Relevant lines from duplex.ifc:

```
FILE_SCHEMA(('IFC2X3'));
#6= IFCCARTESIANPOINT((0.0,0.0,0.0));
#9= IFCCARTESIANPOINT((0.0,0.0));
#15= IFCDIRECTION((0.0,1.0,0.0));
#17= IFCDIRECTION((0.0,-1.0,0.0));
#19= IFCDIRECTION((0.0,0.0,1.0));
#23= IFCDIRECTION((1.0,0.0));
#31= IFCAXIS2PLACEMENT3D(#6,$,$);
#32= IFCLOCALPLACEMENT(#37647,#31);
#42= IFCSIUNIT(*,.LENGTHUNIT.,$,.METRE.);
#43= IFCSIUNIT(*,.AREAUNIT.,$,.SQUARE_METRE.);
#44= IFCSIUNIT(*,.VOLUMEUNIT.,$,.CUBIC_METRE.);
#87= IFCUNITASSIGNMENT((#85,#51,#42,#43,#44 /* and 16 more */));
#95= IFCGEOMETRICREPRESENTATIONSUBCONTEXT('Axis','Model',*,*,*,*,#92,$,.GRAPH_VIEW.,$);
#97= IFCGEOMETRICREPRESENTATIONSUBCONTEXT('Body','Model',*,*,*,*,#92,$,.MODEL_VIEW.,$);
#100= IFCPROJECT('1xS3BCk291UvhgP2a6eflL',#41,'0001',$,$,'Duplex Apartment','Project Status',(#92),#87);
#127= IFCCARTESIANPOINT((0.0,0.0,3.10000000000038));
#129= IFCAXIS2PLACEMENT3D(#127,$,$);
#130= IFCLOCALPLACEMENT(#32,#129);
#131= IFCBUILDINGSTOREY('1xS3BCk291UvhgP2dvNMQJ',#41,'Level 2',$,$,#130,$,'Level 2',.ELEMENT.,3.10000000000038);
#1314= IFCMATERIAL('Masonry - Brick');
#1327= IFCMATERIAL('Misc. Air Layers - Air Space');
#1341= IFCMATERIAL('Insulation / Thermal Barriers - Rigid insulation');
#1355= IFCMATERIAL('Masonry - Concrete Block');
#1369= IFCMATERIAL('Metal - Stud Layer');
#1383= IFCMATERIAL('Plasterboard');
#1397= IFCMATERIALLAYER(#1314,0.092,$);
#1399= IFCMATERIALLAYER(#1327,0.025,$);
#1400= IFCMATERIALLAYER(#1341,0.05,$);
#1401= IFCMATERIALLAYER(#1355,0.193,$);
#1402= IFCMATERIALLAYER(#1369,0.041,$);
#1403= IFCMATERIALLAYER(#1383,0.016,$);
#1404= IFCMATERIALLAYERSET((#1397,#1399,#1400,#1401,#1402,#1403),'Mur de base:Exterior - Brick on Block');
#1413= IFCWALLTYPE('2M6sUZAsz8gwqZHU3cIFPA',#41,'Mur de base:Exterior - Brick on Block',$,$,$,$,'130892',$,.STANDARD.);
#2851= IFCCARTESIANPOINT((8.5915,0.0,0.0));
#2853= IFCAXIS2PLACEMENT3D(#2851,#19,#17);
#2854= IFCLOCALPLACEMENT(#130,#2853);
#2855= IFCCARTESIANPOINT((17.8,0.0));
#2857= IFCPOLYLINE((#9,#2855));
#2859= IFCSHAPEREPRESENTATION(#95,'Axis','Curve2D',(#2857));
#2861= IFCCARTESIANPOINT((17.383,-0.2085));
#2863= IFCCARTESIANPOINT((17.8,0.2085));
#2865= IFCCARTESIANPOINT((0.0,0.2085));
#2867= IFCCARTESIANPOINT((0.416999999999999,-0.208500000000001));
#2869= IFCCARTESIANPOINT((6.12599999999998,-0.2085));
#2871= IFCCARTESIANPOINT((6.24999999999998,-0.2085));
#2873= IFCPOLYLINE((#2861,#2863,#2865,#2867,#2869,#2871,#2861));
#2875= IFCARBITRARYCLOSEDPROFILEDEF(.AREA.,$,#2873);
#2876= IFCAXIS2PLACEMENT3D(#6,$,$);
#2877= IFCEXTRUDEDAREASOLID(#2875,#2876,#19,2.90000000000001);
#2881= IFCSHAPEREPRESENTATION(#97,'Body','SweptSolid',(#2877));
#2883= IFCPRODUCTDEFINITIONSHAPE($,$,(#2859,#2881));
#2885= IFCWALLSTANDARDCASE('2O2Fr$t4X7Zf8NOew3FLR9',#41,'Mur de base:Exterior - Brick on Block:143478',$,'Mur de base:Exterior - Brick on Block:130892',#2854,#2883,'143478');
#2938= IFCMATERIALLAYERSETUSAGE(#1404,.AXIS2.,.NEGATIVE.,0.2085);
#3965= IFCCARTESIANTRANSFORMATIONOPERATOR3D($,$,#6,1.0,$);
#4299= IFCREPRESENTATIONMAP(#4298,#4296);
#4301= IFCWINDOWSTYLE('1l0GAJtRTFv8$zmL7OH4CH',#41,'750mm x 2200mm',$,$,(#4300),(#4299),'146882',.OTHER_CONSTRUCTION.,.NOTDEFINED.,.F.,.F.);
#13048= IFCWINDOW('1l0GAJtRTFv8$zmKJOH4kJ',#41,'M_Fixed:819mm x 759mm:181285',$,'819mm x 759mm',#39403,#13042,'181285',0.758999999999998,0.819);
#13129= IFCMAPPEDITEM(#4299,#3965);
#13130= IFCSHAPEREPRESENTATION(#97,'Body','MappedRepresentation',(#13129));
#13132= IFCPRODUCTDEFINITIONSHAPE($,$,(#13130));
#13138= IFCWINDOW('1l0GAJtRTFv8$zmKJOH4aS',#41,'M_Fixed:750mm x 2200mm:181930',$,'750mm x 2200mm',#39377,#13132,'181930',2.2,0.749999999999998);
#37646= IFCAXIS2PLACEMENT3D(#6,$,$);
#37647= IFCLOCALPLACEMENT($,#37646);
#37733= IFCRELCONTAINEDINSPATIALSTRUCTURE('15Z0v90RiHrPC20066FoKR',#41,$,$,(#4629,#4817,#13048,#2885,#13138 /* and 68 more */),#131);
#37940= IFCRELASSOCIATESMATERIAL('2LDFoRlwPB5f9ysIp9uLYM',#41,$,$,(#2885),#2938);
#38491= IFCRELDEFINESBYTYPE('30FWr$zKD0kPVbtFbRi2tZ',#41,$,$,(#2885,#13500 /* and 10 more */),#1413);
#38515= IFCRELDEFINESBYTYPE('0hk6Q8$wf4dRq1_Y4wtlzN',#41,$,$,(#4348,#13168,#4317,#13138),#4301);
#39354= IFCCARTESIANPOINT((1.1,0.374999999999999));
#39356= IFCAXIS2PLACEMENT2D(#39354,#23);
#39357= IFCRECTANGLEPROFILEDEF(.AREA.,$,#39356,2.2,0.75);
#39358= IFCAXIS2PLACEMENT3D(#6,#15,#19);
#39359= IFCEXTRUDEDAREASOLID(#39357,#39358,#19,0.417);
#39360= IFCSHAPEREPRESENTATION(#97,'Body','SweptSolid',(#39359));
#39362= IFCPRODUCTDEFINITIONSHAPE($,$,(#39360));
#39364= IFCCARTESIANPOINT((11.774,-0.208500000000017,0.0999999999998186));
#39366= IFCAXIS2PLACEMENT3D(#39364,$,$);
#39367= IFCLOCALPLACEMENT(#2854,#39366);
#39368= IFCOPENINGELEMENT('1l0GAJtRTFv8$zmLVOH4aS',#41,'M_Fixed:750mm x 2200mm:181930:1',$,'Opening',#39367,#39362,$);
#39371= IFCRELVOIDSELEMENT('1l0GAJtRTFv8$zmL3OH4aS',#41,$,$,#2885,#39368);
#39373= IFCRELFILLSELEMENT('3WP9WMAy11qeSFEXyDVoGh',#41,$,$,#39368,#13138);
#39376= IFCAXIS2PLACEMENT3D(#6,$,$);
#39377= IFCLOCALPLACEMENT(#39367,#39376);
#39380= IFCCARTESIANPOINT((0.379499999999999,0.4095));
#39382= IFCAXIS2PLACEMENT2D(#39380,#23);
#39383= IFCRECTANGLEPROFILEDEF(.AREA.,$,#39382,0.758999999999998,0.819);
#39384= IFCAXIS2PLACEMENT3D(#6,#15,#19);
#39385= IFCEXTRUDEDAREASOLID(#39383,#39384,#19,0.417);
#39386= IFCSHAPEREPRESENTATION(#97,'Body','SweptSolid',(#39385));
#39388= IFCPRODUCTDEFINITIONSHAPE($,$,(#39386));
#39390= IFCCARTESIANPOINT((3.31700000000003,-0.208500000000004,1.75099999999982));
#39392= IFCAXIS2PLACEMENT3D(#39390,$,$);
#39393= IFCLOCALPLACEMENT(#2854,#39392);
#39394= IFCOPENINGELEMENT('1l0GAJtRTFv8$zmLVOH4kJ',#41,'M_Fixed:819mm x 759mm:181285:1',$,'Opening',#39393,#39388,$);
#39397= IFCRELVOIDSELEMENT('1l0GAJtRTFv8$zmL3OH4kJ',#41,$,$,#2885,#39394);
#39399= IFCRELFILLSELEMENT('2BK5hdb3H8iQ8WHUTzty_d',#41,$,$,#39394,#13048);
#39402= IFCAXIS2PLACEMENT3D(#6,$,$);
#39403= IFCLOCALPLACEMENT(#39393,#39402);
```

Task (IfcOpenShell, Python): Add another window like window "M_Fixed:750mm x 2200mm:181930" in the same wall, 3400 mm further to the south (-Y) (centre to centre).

```python
import ifcopenshell
import ifcopenshell.api.feature
import ifcopenshell.api.geometry
import ifcopenshell.api.root
import ifcopenshell.geom
import ifcopenshell.util.element
import ifcopenshell.util.placement
import ifcopenshell.util.shape

model = ifcopenshell.open("duplex.ifc")
settings = ifcopenshell.geom.settings()


def volume(element):
    """Net volume in cubic metres, openings subtracted."""
    shape = ifcopenshell.geom.create_shape(settings, element)
    return ifcopenshell.util.shape.get_volume(shape.geometry)


def reuse_history(source, copy):
    """copy_class also copies each property set's owner history, people and application; keep the originals."""
    for rel in copy.IsDefinedBy:
        if rel.is_a("IfcRelDefinesByProperties") and (history := rel.RelatingPropertyDefinition.OwnerHistory):
            rel.RelatingPropertyDefinition.OwnerHistory = source.OwnerHistory
            ifcopenshell.util.element.remove_deep2(model, history)


window = model.by_guid("1l0GAJtRTFv8$zmKJOH4aS")
opening = window.FillsVoids[0].RelatingOpeningElement
wall = opening.VoidsElements[0].RelatingBuildingElement
before = volume(wall)
shift = ifcopenshell.util.placement.get_local_placement(wall.ObjectPlacement)[:3, 0] * 3.4

# copy_class copies the void relationship, type, container and properties, but no geometry.
new_opening = ifcopenshell.api.root.copy_class(model, product=opening)
new_opening.Representation = ifcopenshell.util.element.copy_deep(
    model, opening.Representation, exclude=["IfcGeometricRepresentationContext", "IfcRepresentationMap"]
)
new_opening.Name = "M_Fixed:750mm x 2200mm"
new_window = ifcopenshell.api.root.copy_class(model, product=window)
new_window.Representation = ifcopenshell.util.element.copy_deep(
    model, window.Representation, exclude=["IfcGeometricRepresentationContext", "IfcRepresentationMap"]
)
new_window.Name = "M_Fixed:750mm x 2200mm"
new_window.Tag = None
reuse_history(window, new_window)
fills = ifcopenshell.api.feature.add_filling(model, opening=new_opening, element=new_window)
fills.OwnerHistory = new_window.OwnerHistory  # required in IFC2X3

for old, new in ((opening, new_opening), (window, new_window)):
    matrix = ifcopenshell.util.placement.get_local_placement(old.ObjectPlacement)
    matrix[:3, 3] += shift
    ifcopenshell.api.geometry.edit_object_placement(model, product=new, matrix=matrix, is_si=False)

after = volume(wall)

print(f"wall volume {before:.3f} -> {after:.3f} m3")

model.write("duplex_edited.ifc")
```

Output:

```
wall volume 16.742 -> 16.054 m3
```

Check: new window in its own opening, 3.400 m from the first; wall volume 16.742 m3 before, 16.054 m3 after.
